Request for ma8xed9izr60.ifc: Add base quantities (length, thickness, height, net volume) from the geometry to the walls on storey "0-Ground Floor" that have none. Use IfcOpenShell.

First a look at what the model holds.

```python
import ifcopenshell
import ifcopenshell.util.element
import ifcopenshell.util.unit

model = ifcopenshell.open("ma8xed9izr60.ifc")
print(model.schema)
for unit_type in ("LENGTHUNIT", "AREAUNIT", "VOLUMEUNIT"):
    print(unit_type, ifcopenshell.util.unit.calculate_unit_scale(model, unit_type))
storey = next(s for s in model.by_type("IfcBuildingStorey") if s.Name == "0-Ground Floor")
walls = [e for e in ifcopenshell.util.element.get_decomposition(storey) if e.is_a("IfcWall")]
for e in sorted(walls, key=lambda e: e.id()):
    print(e.id(), e.is_a(), e.Name, list(ifcopenshell.util.element.get_psets(e, qtos_only=True)), sep=" | ")
```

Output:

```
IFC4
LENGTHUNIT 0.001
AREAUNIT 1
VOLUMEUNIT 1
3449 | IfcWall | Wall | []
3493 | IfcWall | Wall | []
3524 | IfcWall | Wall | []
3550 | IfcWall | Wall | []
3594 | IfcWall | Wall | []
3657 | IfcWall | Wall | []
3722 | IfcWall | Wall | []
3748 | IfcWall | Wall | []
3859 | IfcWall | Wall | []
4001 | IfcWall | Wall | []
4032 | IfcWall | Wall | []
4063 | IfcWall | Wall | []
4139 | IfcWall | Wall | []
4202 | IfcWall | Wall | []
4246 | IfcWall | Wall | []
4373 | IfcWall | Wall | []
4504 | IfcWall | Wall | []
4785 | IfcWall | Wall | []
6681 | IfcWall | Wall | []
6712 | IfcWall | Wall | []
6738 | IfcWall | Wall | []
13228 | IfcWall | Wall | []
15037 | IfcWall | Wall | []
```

```python
import ifcopenshell
import ifcopenshell.api.pset
import ifcopenshell.geom
import ifcopenshell.util.element
import ifcopenshell.util.shape
import ifcopenshell.util.unit

model = ifcopenshell.open("ma8xed9izr60.ifc")
unit_scale = ifcopenshell.util.unit.calculate_unit_scale(model)
volume_scale = ifcopenshell.util.unit.calculate_unit_scale(model, "VOLUMEUNIT")
settings = ifcopenshell.geom.settings()

storey = next(s for s in model.by_type("IfcBuildingStorey") if s.Name == "0-Ground Floor")
walls = [e for e in ifcopenshell.util.element.get_decomposition(storey) if e.is_a("IfcWall")]

for e in sorted(walls, key=lambda e: e.id()):
    if ifcopenshell.util.element.get_psets(e, qtos_only=True, should_inherit=False):
        continue
    # Geometry comes back in metres, in the element's own axes.
    shape = ifcopenshell.geom.create_shape(settings, e)
    values = {
        "Length": ifcopenshell.util.shape.get_x(shape.geometry) / unit_scale,
        "Width": ifcopenshell.util.shape.get_y(shape.geometry) / unit_scale,
        "Height": ifcopenshell.util.shape.get_z(shape.geometry) / unit_scale,
        "NetVolume": ifcopenshell.util.shape.get_volume(shape.geometry) / volume_scale,
    }
    qto = ifcopenshell.api.pset.add_qto(model, product=e, name="Qto_WallBaseQuantities")
    ifcopenshell.api.pset.edit_qto(model, qto=qto, properties=values)
    print(e.id(), {k: round(v, 3) for k, v in values.items()})

model.write("ma8xed9izr60_v2.ifc")
```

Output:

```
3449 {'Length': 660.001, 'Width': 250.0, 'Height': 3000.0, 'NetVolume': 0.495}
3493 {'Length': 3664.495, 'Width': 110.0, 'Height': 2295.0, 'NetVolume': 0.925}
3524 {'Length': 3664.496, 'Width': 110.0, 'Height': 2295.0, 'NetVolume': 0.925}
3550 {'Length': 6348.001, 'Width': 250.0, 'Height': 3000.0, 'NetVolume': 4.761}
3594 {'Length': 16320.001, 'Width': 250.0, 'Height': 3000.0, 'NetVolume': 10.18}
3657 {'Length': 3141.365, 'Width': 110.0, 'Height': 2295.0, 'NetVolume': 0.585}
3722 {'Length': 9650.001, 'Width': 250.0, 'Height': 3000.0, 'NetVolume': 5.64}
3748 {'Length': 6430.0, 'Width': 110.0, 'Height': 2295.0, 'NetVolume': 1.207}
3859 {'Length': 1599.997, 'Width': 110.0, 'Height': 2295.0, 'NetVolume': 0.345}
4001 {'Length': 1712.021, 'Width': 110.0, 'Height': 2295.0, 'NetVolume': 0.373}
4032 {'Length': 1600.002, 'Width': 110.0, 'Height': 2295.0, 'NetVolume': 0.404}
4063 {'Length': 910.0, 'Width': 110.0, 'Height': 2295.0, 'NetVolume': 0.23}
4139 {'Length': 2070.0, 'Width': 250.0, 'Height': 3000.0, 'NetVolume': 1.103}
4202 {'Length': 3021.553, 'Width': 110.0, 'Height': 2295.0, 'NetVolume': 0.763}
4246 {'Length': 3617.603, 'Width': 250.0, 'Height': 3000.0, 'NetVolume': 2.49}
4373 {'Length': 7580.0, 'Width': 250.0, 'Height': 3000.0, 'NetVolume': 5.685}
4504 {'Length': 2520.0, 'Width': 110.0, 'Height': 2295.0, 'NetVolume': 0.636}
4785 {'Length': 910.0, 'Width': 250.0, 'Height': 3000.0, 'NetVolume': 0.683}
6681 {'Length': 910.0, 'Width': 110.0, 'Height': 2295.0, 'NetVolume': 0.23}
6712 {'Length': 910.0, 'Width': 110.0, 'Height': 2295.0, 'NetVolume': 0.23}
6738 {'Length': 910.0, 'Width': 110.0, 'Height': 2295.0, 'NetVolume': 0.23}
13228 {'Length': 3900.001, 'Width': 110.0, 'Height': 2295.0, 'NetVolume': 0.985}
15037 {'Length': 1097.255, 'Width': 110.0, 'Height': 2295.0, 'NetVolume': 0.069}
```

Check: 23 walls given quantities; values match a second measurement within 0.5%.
